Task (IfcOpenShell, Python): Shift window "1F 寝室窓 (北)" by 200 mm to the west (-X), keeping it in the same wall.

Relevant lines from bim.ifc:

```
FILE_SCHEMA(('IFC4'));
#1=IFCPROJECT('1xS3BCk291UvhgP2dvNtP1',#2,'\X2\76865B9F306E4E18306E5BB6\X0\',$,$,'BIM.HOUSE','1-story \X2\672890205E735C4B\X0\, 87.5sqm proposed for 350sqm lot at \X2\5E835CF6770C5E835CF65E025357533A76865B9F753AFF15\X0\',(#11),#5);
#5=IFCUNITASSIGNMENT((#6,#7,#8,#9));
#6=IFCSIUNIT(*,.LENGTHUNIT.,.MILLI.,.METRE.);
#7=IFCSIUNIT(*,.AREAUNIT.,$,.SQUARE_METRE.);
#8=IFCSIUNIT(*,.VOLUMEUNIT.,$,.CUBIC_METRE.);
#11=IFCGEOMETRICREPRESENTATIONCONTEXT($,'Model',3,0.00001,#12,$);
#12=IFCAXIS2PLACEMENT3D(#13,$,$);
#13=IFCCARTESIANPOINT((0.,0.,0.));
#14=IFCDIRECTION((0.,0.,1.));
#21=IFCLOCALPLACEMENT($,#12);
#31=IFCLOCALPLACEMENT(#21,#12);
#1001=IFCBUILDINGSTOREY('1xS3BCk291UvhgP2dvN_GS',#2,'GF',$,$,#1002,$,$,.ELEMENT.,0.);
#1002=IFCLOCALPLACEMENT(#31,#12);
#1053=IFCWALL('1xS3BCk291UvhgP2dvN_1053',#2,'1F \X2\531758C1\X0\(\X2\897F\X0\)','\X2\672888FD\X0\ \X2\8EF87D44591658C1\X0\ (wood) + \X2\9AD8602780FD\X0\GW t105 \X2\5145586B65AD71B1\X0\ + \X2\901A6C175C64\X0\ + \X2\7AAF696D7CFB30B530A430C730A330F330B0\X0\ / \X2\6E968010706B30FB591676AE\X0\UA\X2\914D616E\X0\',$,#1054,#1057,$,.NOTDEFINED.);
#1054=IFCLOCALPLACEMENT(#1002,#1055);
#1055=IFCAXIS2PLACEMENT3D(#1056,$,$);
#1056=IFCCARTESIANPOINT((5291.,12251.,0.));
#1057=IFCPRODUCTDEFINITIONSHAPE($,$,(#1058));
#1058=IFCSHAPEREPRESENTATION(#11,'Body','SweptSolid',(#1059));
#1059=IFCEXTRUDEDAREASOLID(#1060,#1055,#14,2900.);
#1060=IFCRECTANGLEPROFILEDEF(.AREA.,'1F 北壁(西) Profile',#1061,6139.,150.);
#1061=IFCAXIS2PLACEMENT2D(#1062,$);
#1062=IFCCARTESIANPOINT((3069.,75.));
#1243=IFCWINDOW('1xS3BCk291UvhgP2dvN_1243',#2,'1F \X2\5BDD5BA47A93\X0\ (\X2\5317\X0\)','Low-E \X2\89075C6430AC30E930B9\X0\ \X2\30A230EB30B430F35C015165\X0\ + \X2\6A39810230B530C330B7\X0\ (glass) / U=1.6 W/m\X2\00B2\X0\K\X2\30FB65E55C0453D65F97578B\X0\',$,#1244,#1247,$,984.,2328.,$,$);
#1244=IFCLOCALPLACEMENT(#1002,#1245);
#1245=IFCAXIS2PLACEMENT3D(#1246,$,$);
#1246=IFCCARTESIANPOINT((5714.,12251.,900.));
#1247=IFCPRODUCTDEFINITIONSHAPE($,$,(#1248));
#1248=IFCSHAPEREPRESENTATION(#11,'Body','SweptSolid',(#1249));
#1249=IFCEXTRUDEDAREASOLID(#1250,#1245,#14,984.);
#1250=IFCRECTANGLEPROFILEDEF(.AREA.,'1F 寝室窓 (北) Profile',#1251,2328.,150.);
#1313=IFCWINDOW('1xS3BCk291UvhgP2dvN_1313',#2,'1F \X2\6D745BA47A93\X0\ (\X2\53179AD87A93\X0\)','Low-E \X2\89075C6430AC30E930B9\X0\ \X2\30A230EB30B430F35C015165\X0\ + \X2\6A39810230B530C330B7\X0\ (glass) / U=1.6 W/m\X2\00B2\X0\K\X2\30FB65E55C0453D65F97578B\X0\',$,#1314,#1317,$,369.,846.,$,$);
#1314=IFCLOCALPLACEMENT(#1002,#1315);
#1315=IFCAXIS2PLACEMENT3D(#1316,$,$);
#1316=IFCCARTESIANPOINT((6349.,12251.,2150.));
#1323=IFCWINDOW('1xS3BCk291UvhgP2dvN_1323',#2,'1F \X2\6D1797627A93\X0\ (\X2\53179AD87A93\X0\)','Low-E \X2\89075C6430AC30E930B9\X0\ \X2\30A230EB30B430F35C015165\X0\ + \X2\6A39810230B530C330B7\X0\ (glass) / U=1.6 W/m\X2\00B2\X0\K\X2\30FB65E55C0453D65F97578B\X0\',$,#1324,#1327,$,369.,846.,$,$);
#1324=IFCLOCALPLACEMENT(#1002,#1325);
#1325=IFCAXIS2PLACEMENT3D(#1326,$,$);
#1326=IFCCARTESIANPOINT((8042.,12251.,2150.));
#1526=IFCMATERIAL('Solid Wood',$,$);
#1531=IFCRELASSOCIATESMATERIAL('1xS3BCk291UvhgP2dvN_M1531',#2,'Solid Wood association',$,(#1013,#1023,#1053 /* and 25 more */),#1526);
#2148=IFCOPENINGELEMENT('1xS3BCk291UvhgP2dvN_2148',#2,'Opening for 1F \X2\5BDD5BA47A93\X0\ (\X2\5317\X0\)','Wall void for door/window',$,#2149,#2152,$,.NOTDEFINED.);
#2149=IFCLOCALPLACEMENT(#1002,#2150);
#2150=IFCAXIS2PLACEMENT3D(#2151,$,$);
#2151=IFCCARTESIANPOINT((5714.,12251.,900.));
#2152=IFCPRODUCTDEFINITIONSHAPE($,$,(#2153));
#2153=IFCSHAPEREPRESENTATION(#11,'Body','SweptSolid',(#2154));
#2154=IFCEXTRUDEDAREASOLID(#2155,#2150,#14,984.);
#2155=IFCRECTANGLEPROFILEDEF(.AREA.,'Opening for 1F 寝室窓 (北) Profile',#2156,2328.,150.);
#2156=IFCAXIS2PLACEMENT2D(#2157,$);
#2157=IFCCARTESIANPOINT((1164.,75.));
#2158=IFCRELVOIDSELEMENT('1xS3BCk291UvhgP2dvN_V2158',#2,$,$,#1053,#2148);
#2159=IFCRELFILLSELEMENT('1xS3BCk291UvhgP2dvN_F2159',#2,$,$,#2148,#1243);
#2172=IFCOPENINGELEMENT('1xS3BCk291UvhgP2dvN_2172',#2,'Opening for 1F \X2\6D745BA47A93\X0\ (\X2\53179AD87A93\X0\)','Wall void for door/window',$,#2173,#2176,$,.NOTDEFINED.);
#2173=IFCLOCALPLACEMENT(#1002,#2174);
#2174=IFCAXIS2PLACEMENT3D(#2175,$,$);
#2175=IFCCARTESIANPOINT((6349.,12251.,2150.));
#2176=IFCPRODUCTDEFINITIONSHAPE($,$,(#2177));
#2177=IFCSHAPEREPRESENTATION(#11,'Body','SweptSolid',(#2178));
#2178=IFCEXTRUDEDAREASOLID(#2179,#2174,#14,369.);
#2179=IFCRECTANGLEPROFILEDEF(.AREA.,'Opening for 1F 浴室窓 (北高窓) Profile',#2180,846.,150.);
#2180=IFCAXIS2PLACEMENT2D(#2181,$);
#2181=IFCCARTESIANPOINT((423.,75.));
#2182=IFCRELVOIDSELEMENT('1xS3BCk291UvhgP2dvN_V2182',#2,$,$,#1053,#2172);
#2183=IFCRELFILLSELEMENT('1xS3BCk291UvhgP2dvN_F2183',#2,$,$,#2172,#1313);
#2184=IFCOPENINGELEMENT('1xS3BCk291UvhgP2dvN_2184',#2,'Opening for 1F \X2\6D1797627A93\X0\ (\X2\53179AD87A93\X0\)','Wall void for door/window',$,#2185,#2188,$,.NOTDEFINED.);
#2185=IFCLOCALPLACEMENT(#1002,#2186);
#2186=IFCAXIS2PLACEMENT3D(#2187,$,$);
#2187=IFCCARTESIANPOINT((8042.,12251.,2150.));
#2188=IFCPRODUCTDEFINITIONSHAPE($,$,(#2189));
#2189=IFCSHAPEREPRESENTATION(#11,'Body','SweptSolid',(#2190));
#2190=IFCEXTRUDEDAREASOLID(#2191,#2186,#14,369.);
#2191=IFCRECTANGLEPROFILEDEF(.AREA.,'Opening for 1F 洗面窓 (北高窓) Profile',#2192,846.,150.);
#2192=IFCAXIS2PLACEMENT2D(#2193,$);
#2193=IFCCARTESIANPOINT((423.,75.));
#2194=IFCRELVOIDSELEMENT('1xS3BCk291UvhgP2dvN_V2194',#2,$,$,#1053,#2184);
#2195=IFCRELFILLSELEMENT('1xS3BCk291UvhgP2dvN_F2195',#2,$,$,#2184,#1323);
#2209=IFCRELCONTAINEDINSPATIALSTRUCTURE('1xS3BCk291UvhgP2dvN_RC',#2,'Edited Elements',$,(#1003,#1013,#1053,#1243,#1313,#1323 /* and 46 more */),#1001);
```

```python
import ifcopenshell
import ifcopenshell.api.geometry
import ifcopenshell.util.placement
import ifcopenshell.util.unit

model = ifcopenshell.open("bim.ifc")
unit_scale = ifcopenshell.util.unit.calculate_unit_scale(model)

window = model.by_id(1243)
opening = window.FillsVoids[0].RelatingOpeningElement
wall = opening.VoidsElements[0].RelatingBuildingElement

wall_matrix = ifcopenshell.util.placement.get_local_placement(wall.ObjectPlacement)
shift = wall_matrix[:3, 0] * -0.2 / unit_scale
before = ifcopenshell.util.placement.get_local_placement(window.ObjectPlacement)[:3, 3].copy()

# The window is not placed relative to its opening, so move both.
for product in (opening, window):
    matrix = ifcopenshell.util.placement.get_local_placement(product.ObjectPlacement)
    matrix[:3, 3] += shift
    ifcopenshell.api.geometry.edit_object_placement(model, product=product, matrix=matrix, is_si=False)

after = ifcopenshell.util.placement.get_local_placement(window.ObjectPlacement)[:3, 3]
print("window moved by", (after - before).round(3) + 0.0)

model.write("bim_v2.ifc")
```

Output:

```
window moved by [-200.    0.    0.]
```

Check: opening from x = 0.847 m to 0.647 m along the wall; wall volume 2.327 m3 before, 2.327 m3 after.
